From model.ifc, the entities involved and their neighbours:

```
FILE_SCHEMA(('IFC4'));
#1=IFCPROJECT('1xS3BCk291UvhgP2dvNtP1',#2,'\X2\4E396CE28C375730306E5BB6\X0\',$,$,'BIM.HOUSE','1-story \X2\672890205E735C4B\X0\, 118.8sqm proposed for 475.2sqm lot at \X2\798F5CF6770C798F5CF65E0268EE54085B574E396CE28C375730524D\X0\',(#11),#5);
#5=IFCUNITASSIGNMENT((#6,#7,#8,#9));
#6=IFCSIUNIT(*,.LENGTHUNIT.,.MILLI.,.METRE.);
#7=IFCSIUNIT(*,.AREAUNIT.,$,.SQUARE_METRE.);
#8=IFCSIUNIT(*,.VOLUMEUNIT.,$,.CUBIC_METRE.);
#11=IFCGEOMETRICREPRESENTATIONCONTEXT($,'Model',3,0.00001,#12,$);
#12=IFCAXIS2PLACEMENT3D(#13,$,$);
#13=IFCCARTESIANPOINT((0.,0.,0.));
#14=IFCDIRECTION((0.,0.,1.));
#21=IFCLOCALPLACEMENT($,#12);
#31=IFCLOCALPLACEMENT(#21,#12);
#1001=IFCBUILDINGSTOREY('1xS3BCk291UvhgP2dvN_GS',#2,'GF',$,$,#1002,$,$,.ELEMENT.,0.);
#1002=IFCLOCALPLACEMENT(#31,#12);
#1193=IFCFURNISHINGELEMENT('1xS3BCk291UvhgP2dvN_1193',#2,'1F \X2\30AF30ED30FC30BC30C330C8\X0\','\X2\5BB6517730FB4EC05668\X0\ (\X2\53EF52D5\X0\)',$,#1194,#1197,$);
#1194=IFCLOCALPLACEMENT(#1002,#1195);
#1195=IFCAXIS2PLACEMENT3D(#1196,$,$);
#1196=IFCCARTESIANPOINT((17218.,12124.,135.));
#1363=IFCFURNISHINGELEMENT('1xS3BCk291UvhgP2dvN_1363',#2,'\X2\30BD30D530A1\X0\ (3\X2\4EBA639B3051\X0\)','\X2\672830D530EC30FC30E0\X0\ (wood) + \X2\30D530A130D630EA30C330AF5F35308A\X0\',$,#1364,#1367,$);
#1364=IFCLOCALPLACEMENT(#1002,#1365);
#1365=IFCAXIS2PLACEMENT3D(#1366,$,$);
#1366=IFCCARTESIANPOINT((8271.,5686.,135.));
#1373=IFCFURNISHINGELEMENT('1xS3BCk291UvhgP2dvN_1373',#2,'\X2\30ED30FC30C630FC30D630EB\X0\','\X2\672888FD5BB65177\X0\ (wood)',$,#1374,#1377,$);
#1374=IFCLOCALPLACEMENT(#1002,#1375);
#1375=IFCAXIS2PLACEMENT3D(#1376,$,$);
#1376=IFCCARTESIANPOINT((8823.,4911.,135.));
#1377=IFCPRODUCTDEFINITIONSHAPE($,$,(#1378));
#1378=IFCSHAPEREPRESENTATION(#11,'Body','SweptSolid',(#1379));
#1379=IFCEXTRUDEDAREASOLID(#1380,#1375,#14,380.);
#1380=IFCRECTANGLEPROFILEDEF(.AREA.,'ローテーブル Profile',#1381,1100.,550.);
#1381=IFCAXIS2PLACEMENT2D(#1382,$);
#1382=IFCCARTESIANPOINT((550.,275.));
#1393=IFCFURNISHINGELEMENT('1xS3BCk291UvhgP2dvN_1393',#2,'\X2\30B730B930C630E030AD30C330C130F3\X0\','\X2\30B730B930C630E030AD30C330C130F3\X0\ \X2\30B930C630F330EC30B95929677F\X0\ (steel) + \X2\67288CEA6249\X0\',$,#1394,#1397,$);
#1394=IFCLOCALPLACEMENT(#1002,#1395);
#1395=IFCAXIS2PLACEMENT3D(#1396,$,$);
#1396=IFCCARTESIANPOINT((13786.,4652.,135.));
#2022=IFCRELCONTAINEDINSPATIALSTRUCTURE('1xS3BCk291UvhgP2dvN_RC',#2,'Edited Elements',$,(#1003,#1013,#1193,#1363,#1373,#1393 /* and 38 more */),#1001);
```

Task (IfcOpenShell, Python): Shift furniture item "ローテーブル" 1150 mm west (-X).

```python
import ifcopenshell
import ifcopenshell.api.geometry
import ifcopenshell.util.placement
import ifcopenshell.util.unit

model = ifcopenshell.open("model.ifc")
unit_scale = ifcopenshell.util.unit.calculate_unit_scale(model)

item = model.by_guid("1xS3BCk291UvhgP2dvN_1373")
matrix = ifcopenshell.util.placement.get_local_placement(item.ObjectPlacement)
matrix[0, 3] -= 1.15 / unit_scale
ifcopenshell.api.geometry.edit_object_placement(model, product=item, matrix=matrix, is_si=False)

print(ifcopenshell.util.placement.get_local_placement(item.ObjectPlacement).round(3) + 0.0)

model.write("model-out.ifc")
```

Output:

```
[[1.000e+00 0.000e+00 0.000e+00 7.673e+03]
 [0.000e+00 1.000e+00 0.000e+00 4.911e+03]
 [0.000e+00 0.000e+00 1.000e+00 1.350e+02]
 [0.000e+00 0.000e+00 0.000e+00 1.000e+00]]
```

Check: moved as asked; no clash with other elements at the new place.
